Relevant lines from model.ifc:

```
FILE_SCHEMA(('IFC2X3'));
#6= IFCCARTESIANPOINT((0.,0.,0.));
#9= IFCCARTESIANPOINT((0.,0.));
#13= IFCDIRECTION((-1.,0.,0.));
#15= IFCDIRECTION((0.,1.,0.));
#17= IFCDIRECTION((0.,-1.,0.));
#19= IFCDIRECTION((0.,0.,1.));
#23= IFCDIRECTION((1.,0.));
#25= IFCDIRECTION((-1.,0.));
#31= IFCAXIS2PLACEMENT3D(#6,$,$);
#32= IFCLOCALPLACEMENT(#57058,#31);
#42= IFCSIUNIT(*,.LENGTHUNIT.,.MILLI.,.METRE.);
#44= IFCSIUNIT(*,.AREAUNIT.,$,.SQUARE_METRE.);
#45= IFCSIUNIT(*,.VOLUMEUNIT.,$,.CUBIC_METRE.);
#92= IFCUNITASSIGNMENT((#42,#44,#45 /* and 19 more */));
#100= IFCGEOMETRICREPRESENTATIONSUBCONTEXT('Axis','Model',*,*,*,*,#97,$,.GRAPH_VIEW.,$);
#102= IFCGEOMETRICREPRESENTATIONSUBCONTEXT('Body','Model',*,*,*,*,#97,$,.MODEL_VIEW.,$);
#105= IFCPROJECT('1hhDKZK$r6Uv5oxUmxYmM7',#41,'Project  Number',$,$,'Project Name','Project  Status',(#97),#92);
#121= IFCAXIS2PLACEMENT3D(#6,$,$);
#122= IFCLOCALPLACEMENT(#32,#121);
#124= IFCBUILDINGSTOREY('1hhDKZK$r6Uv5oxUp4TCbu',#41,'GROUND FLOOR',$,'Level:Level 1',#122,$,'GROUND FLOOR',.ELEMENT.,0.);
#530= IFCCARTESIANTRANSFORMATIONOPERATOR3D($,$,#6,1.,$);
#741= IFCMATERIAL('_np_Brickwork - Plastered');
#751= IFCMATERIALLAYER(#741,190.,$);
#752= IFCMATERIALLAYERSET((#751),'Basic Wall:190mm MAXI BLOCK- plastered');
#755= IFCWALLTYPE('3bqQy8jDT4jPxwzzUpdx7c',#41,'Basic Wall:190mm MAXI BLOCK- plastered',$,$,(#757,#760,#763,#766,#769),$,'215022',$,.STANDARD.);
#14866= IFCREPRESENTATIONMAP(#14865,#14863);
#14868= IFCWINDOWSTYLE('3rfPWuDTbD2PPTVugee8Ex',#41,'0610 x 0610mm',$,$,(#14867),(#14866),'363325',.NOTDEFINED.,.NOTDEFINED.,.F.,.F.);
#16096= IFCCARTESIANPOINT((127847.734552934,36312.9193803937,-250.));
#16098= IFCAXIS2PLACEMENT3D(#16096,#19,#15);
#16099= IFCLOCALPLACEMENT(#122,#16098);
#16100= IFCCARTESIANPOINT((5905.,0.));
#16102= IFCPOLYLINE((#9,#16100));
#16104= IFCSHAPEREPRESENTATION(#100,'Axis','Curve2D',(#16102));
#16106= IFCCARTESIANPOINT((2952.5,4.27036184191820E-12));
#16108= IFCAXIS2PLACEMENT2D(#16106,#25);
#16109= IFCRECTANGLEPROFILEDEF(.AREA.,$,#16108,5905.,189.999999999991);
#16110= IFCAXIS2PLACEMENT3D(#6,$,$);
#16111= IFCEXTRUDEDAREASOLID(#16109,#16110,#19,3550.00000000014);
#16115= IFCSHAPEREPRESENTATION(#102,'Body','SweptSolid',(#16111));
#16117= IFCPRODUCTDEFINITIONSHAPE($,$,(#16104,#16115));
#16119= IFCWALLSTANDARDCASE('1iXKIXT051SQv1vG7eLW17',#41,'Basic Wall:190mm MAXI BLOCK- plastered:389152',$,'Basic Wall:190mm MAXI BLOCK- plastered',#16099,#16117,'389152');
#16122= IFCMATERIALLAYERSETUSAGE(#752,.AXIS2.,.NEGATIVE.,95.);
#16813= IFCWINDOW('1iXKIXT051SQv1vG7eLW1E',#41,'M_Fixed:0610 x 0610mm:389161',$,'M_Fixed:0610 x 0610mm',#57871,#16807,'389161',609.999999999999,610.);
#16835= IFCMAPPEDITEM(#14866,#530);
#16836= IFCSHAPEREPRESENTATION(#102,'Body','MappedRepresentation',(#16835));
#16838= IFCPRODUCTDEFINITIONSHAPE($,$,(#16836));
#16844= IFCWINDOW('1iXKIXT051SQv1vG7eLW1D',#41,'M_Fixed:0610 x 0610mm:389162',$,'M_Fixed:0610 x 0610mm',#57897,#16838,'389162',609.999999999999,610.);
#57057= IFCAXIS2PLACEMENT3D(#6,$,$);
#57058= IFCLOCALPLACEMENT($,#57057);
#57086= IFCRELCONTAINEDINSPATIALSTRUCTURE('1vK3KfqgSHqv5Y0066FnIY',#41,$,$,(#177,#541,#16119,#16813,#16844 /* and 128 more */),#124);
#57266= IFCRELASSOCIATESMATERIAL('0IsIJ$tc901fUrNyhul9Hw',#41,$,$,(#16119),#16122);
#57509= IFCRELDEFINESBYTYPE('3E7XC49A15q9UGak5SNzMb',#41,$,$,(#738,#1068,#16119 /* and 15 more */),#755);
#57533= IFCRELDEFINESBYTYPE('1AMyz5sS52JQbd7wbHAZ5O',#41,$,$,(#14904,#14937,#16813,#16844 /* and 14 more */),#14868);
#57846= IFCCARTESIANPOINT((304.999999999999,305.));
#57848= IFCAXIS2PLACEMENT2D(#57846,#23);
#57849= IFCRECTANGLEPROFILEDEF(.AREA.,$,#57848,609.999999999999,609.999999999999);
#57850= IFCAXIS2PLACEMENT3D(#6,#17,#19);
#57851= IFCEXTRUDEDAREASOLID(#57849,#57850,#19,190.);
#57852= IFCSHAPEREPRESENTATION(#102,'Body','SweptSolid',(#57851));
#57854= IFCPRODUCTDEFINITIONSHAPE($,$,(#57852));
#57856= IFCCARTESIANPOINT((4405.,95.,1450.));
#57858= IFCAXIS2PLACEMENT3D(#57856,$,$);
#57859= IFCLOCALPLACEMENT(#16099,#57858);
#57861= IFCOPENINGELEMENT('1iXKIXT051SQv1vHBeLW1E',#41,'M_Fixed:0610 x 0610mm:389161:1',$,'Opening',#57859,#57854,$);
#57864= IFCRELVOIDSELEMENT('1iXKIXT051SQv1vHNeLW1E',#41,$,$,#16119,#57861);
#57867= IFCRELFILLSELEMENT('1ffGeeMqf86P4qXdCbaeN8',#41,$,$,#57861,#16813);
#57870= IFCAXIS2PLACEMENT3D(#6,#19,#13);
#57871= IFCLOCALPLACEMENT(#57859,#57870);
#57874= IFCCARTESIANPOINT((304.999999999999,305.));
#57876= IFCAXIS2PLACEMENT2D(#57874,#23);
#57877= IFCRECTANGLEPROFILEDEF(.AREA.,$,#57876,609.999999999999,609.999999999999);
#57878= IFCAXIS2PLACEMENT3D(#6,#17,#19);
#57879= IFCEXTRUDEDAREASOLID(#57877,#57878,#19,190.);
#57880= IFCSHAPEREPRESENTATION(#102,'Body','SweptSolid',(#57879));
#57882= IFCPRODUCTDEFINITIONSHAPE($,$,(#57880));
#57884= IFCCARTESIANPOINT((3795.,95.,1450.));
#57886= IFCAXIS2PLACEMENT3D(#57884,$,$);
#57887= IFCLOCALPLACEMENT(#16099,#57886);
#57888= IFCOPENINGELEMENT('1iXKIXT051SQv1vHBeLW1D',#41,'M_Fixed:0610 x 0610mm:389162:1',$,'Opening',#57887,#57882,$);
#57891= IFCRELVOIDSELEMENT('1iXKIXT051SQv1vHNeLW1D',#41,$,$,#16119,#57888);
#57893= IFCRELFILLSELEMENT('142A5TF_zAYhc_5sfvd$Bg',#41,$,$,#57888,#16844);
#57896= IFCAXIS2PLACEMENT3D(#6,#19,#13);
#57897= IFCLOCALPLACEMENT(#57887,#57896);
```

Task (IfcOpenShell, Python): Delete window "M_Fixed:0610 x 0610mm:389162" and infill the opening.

```python
import ifcopenshell
import ifcopenshell.api.feature
import ifcopenshell.api.root
import ifcopenshell.geom
import ifcopenshell.util.shape

model = ifcopenshell.open("model.ifc")
settings = ifcopenshell.geom.settings()


def volume(element):
    """Net volume in cubic metres, openings subtracted."""
    shape = ifcopenshell.geom.create_shape(settings, element)
    return ifcopenshell.util.shape.get_volume(shape.geometry)


window = model.by_id(16844)
opening = window.FillsVoids[0].RelatingOpeningElement
wall = opening.VoidsElements[0].RelatingBuildingElement
before = volume(wall)

ifcopenshell.api.root.remove_product(model, product=window)
ifcopenshell.api.feature.remove_feature(model, feature=opening)

after = volume(wall)

print(f"wall volume {before:.3f} -> {after:.3f} m3")

model.write("model_edited.ifc")
```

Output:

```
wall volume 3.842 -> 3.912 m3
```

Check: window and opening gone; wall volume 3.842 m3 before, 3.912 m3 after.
